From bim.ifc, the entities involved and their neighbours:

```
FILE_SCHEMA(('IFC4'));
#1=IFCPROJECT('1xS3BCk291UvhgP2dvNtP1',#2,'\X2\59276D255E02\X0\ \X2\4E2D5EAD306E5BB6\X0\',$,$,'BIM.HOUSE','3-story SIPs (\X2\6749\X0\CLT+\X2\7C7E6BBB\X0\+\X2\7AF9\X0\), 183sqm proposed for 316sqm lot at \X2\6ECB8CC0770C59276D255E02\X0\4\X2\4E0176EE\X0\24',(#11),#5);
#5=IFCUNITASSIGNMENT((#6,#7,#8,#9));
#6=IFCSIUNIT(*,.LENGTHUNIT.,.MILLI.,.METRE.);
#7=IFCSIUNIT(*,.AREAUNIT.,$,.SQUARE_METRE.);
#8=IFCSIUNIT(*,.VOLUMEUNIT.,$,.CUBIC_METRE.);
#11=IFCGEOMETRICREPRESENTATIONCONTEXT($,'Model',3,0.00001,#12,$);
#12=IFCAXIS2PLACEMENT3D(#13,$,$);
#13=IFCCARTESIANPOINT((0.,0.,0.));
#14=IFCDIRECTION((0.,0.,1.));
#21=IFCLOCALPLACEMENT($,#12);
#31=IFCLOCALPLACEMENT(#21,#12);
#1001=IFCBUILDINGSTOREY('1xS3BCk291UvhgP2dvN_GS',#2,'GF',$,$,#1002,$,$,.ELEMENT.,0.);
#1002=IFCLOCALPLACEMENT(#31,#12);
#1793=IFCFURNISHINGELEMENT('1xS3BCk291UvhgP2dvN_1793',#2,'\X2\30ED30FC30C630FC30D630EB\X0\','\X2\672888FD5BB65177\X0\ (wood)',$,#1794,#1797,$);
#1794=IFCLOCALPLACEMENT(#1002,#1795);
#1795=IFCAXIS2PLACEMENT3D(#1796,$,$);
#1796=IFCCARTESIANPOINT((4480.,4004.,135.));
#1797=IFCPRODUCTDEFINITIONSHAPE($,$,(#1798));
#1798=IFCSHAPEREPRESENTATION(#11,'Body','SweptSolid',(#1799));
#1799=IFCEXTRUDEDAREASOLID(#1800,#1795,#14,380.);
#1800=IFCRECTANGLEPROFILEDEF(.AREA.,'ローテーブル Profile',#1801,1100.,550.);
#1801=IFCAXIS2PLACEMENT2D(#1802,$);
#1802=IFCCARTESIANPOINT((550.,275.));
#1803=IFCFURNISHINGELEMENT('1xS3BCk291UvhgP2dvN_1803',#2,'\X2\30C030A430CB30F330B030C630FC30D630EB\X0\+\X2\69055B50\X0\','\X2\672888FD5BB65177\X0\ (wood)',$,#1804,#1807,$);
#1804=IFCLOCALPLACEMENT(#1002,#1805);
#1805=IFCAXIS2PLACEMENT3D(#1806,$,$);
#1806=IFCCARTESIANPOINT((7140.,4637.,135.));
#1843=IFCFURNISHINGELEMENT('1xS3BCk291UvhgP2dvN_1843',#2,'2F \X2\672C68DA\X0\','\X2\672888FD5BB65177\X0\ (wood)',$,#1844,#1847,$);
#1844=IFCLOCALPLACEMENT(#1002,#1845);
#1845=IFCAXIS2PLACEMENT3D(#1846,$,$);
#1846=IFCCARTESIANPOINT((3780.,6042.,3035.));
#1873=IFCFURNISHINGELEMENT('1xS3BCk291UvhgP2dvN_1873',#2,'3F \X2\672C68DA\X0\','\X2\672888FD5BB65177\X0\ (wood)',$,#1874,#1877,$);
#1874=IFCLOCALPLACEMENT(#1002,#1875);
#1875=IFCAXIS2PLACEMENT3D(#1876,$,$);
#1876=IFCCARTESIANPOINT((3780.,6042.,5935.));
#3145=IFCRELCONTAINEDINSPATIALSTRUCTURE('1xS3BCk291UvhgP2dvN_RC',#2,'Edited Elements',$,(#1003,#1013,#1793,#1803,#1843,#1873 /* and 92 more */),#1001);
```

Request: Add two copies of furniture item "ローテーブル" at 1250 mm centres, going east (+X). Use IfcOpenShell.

```python
import numpy as np
import ifcopenshell
import ifcopenshell.api.geometry
import ifcopenshell.api.root
import ifcopenshell.util.element
import ifcopenshell.util.placement

model = ifcopenshell.open("bim.ifc")


def reuse_history(source, copy):
    """copy_class also copies each property set's owner history, people and application; keep the originals."""
    for rel in copy.IsDefinedBy:
        if rel.is_a("IfcRelDefinesByProperties") and (history := rel.RelatingPropertyDefinition.OwnerHistory):
            rel.RelatingPropertyDefinition.OwnerHistory = source.OwnerHistory
            ifcopenshell.util.element.remove_deep2(model, history)


source = model.by_id(1793)
base = ifcopenshell.util.placement.get_local_placement(source.ObjectPlacement)
step = np.array([1.0, 0.0, 0.0]) * 1250.0

for i in range(1, 3):
    copy = ifcopenshell.api.root.copy_class(model, product=source)
    copy.Representation = ifcopenshell.util.element.copy_deep(
        model, source.Representation, exclude=["IfcGeometricRepresentationContext", "IfcRepresentationMap"]
    )
    reuse_history(source, copy)
    matrix = base.copy()
    matrix[:3, 3] += i * step
    print("added at", matrix[:3, 3].round(3) + 0.0)
    ifcopenshell.api.geometry.edit_object_placement(model, product=copy, matrix=matrix, is_si=False)

model.write("bim_rev.ifc")
```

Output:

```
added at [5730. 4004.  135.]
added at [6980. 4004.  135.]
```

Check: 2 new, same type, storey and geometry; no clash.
